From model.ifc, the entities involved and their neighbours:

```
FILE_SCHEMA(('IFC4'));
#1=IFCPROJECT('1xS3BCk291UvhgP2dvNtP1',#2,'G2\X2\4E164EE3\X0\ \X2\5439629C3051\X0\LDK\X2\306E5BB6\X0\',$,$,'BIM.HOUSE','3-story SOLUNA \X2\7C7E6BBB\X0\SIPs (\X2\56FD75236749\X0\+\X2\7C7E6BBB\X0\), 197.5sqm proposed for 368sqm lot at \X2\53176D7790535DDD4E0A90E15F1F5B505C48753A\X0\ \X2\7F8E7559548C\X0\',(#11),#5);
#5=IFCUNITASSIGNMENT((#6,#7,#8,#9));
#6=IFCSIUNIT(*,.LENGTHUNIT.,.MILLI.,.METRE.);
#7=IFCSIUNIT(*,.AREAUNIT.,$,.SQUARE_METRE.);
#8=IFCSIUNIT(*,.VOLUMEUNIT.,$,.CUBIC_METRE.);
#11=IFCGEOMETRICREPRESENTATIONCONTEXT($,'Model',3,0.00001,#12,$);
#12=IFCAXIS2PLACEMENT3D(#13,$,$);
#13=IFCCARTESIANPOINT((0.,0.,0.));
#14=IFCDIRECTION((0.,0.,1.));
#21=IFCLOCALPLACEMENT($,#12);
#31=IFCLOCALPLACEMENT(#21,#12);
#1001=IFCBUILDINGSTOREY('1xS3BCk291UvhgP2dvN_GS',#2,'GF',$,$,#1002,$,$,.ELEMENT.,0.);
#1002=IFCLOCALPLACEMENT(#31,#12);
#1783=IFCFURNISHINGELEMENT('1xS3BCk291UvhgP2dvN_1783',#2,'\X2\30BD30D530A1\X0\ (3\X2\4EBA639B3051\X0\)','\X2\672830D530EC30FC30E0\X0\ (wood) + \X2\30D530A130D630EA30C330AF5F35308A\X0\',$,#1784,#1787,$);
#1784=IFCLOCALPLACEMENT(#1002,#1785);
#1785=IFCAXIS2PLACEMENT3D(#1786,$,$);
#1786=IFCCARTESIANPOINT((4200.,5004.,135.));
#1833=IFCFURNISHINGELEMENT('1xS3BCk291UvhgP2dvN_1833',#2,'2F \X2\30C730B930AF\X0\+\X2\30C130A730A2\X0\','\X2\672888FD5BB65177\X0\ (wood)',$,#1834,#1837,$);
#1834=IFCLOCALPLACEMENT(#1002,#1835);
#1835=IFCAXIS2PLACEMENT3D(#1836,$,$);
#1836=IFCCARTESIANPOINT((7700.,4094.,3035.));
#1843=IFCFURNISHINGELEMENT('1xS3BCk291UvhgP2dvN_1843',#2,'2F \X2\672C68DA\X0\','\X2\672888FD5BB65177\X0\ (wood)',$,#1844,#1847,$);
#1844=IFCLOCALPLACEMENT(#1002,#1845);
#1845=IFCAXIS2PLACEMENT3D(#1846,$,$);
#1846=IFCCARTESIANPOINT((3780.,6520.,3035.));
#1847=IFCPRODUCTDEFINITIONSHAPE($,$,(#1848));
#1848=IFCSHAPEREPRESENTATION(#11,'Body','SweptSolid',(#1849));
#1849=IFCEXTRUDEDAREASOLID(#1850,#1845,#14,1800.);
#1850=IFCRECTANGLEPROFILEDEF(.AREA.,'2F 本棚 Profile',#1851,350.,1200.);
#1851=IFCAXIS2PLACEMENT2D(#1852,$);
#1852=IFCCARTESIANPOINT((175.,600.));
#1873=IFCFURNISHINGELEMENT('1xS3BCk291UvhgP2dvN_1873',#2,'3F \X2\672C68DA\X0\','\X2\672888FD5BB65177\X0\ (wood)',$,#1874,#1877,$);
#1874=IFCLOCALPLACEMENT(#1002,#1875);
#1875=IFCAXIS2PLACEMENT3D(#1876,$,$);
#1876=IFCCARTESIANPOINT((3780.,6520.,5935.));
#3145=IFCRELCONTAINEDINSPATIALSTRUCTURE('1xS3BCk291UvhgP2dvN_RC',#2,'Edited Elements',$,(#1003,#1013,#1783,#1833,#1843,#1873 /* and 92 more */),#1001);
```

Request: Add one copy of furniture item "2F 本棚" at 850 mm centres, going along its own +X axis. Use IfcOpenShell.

```python
import ifcopenshell
import ifcopenshell.api.geometry
import ifcopenshell.api.root
import ifcopenshell.util.element
import ifcopenshell.util.placement
import ifcopenshell.util.unit

model = ifcopenshell.open("model.ifc")
unit_scale = ifcopenshell.util.unit.calculate_unit_scale(model)


def reuse_history(source, copy):
    """copy_class also copies each property set's owner history, people and application; keep the originals."""
    for rel in copy.IsDefinedBy:
        if rel.is_a("IfcRelDefinesByProperties") and (history := rel.RelatingPropertyDefinition.OwnerHistory):
            rel.RelatingPropertyDefinition.OwnerHistory = source.OwnerHistory
            ifcopenshell.util.element.remove_deep2(model, history)


source = model.by_guid("1xS3BCk291UvhgP2dvN_1843")
base = ifcopenshell.util.placement.get_local_placement(source.ObjectPlacement)
step = base[:3, 0] * 0.85 / unit_scale

for i in range(1, 2):
    copy = ifcopenshell.api.root.copy_class(model, product=source)
    copy.Representation = ifcopenshell.util.element.copy_deep(
        model, source.Representation, exclude=["IfcGeometricRepresentationContext", "IfcRepresentationMap"]
    )
    reuse_history(source, copy)
    matrix = base.copy()
    matrix[:3, 3] += i * step
    print("added at", matrix[:3, 3].round(3) + 0.0)
    ifcopenshell.api.geometry.edit_object_placement(model, product=copy, matrix=matrix, is_si=False)

model.write("model_rev.ifc")
```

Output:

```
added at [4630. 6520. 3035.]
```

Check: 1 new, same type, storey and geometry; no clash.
